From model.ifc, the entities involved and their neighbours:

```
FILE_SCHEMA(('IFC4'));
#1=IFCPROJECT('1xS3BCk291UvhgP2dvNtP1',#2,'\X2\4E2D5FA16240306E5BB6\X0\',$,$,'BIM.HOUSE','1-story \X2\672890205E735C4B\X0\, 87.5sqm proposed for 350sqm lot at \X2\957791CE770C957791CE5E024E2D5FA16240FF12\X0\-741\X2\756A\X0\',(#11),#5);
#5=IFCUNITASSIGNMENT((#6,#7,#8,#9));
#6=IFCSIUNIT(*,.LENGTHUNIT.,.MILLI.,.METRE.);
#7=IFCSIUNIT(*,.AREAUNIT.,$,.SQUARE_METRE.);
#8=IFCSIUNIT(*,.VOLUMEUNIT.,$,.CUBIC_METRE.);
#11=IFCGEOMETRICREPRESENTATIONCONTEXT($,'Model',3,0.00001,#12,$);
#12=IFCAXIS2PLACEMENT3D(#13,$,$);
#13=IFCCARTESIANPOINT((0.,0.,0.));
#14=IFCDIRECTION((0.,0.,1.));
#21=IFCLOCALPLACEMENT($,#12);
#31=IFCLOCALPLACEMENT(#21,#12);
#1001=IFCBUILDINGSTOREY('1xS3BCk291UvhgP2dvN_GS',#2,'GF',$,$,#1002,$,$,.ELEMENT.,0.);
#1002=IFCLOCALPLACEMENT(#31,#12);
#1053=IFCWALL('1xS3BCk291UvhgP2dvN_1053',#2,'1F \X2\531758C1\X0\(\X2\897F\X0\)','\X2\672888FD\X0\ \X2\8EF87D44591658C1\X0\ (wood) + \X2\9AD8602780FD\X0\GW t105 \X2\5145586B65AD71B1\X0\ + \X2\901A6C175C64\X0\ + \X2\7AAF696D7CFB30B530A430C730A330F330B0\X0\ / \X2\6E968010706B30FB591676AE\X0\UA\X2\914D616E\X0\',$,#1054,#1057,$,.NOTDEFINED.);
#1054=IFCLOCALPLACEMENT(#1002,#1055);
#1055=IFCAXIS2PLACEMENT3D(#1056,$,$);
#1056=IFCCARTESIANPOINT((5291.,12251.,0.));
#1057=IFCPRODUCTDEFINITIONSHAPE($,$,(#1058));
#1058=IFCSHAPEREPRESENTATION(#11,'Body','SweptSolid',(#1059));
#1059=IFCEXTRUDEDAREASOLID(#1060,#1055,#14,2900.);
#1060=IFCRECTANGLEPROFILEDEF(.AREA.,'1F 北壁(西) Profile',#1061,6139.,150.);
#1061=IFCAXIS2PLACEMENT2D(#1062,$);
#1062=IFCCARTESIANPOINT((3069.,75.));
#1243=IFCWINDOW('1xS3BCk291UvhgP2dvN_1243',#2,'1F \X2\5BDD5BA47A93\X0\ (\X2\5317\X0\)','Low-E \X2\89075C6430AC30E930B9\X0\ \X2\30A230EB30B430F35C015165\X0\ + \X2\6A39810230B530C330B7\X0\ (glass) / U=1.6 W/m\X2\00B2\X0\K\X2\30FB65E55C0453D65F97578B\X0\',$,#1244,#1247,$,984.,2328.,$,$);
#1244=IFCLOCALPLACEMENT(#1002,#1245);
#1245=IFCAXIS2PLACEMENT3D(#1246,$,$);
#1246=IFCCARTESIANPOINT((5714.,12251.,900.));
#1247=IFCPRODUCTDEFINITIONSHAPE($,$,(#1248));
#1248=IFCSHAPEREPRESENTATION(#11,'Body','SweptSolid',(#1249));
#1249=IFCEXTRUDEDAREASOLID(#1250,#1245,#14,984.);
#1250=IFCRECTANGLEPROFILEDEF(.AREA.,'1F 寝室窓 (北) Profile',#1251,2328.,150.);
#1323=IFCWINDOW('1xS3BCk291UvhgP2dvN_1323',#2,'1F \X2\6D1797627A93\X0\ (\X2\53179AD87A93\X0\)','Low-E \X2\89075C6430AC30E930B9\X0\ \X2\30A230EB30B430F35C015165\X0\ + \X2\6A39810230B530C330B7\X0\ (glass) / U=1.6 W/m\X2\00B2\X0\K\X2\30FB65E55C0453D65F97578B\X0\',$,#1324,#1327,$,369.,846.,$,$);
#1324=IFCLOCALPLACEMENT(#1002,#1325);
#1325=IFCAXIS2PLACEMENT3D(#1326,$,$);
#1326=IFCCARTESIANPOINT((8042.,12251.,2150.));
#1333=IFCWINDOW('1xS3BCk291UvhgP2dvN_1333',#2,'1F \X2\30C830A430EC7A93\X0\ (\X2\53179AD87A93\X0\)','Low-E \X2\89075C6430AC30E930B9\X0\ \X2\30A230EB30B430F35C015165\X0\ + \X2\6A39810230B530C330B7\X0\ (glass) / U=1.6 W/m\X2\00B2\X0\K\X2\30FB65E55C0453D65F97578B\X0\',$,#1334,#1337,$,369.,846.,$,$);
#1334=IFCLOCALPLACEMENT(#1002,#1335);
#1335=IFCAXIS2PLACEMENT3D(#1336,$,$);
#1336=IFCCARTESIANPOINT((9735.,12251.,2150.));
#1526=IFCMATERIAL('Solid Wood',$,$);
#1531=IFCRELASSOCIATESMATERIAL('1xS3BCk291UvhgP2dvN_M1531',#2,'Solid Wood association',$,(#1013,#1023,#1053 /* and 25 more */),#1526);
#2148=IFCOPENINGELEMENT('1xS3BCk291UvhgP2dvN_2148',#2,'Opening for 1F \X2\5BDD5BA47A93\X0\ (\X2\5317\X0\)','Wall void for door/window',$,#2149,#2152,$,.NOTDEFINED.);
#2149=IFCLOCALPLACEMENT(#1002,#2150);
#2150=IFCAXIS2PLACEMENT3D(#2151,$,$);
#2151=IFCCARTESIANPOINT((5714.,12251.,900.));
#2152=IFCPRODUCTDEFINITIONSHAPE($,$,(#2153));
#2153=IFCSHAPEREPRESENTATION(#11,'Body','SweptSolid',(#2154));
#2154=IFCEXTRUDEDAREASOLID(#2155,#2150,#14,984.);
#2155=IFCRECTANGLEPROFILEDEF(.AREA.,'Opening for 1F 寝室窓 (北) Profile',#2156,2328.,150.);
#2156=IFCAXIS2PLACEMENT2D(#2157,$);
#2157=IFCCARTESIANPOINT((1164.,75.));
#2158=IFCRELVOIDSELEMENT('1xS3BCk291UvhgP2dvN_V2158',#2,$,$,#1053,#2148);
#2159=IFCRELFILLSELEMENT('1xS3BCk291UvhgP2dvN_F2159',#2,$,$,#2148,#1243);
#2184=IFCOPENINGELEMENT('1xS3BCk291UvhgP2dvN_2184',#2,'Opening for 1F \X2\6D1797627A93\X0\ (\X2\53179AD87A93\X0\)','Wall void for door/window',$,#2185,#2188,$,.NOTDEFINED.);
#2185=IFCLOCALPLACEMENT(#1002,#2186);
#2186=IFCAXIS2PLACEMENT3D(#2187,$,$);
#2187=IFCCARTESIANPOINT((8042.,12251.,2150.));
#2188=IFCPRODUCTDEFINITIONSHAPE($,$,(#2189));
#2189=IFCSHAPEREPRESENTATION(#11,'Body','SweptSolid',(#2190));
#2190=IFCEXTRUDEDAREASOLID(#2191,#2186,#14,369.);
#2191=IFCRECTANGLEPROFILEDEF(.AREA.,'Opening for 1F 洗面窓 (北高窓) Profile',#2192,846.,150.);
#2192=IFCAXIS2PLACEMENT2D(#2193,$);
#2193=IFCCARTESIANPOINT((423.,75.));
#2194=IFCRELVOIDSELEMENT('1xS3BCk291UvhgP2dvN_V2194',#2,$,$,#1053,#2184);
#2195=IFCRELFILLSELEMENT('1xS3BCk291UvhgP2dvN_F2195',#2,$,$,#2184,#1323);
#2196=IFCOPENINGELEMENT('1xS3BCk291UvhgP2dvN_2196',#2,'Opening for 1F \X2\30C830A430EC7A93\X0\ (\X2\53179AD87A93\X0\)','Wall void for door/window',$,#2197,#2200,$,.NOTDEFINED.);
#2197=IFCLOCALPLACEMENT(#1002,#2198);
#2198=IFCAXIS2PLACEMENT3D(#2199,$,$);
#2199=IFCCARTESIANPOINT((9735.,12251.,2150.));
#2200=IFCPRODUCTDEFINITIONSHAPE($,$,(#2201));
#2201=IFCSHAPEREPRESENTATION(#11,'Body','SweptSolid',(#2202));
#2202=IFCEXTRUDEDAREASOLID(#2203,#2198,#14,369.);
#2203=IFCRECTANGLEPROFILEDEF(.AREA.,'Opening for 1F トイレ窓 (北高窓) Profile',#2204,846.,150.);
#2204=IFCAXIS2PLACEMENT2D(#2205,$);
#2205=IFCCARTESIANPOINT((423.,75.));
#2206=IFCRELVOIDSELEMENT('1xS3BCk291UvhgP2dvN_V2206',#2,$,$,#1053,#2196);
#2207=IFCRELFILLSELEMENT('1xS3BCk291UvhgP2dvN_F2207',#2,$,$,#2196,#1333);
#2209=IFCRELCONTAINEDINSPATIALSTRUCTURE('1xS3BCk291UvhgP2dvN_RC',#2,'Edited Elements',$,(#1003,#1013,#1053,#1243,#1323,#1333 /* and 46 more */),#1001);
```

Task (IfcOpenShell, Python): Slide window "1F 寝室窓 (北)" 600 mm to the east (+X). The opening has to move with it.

```python
import ifcopenshell
import ifcopenshell.api.geometry
import ifcopenshell.util.placement
import ifcopenshell.util.unit

model = ifcopenshell.open("model.ifc")
unit_scale = ifcopenshell.util.unit.calculate_unit_scale(model)

window = model.by_guid("1xS3BCk291UvhgP2dvN_1243")
opening = window.FillsVoids[0].RelatingOpeningElement
wall = opening.VoidsElements[0].RelatingBuildingElement

wall_matrix = ifcopenshell.util.placement.get_local_placement(wall.ObjectPlacement)
shift = wall_matrix[:3, 0] * 0.6 / unit_scale
before = ifcopenshell.util.placement.get_local_placement(window.ObjectPlacement)[:3, 3].copy()

# The window is not placed relative to its opening, so move both.
for product in (opening, window):
    matrix = ifcopenshell.util.placement.get_local_placement(product.ObjectPlacement)
    matrix[:3, 3] += shift
    ifcopenshell.api.geometry.edit_object_placement(model, product=product, matrix=matrix, is_si=False)

after = ifcopenshell.util.placement.get_local_placement(window.ObjectPlacement)[:3, 3]
print("window moved by", (after - before).round(3) + 0.0)

model.write("model_edited.ifc")
```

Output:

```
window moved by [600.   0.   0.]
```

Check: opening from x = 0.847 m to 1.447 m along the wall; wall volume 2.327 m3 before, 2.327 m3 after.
